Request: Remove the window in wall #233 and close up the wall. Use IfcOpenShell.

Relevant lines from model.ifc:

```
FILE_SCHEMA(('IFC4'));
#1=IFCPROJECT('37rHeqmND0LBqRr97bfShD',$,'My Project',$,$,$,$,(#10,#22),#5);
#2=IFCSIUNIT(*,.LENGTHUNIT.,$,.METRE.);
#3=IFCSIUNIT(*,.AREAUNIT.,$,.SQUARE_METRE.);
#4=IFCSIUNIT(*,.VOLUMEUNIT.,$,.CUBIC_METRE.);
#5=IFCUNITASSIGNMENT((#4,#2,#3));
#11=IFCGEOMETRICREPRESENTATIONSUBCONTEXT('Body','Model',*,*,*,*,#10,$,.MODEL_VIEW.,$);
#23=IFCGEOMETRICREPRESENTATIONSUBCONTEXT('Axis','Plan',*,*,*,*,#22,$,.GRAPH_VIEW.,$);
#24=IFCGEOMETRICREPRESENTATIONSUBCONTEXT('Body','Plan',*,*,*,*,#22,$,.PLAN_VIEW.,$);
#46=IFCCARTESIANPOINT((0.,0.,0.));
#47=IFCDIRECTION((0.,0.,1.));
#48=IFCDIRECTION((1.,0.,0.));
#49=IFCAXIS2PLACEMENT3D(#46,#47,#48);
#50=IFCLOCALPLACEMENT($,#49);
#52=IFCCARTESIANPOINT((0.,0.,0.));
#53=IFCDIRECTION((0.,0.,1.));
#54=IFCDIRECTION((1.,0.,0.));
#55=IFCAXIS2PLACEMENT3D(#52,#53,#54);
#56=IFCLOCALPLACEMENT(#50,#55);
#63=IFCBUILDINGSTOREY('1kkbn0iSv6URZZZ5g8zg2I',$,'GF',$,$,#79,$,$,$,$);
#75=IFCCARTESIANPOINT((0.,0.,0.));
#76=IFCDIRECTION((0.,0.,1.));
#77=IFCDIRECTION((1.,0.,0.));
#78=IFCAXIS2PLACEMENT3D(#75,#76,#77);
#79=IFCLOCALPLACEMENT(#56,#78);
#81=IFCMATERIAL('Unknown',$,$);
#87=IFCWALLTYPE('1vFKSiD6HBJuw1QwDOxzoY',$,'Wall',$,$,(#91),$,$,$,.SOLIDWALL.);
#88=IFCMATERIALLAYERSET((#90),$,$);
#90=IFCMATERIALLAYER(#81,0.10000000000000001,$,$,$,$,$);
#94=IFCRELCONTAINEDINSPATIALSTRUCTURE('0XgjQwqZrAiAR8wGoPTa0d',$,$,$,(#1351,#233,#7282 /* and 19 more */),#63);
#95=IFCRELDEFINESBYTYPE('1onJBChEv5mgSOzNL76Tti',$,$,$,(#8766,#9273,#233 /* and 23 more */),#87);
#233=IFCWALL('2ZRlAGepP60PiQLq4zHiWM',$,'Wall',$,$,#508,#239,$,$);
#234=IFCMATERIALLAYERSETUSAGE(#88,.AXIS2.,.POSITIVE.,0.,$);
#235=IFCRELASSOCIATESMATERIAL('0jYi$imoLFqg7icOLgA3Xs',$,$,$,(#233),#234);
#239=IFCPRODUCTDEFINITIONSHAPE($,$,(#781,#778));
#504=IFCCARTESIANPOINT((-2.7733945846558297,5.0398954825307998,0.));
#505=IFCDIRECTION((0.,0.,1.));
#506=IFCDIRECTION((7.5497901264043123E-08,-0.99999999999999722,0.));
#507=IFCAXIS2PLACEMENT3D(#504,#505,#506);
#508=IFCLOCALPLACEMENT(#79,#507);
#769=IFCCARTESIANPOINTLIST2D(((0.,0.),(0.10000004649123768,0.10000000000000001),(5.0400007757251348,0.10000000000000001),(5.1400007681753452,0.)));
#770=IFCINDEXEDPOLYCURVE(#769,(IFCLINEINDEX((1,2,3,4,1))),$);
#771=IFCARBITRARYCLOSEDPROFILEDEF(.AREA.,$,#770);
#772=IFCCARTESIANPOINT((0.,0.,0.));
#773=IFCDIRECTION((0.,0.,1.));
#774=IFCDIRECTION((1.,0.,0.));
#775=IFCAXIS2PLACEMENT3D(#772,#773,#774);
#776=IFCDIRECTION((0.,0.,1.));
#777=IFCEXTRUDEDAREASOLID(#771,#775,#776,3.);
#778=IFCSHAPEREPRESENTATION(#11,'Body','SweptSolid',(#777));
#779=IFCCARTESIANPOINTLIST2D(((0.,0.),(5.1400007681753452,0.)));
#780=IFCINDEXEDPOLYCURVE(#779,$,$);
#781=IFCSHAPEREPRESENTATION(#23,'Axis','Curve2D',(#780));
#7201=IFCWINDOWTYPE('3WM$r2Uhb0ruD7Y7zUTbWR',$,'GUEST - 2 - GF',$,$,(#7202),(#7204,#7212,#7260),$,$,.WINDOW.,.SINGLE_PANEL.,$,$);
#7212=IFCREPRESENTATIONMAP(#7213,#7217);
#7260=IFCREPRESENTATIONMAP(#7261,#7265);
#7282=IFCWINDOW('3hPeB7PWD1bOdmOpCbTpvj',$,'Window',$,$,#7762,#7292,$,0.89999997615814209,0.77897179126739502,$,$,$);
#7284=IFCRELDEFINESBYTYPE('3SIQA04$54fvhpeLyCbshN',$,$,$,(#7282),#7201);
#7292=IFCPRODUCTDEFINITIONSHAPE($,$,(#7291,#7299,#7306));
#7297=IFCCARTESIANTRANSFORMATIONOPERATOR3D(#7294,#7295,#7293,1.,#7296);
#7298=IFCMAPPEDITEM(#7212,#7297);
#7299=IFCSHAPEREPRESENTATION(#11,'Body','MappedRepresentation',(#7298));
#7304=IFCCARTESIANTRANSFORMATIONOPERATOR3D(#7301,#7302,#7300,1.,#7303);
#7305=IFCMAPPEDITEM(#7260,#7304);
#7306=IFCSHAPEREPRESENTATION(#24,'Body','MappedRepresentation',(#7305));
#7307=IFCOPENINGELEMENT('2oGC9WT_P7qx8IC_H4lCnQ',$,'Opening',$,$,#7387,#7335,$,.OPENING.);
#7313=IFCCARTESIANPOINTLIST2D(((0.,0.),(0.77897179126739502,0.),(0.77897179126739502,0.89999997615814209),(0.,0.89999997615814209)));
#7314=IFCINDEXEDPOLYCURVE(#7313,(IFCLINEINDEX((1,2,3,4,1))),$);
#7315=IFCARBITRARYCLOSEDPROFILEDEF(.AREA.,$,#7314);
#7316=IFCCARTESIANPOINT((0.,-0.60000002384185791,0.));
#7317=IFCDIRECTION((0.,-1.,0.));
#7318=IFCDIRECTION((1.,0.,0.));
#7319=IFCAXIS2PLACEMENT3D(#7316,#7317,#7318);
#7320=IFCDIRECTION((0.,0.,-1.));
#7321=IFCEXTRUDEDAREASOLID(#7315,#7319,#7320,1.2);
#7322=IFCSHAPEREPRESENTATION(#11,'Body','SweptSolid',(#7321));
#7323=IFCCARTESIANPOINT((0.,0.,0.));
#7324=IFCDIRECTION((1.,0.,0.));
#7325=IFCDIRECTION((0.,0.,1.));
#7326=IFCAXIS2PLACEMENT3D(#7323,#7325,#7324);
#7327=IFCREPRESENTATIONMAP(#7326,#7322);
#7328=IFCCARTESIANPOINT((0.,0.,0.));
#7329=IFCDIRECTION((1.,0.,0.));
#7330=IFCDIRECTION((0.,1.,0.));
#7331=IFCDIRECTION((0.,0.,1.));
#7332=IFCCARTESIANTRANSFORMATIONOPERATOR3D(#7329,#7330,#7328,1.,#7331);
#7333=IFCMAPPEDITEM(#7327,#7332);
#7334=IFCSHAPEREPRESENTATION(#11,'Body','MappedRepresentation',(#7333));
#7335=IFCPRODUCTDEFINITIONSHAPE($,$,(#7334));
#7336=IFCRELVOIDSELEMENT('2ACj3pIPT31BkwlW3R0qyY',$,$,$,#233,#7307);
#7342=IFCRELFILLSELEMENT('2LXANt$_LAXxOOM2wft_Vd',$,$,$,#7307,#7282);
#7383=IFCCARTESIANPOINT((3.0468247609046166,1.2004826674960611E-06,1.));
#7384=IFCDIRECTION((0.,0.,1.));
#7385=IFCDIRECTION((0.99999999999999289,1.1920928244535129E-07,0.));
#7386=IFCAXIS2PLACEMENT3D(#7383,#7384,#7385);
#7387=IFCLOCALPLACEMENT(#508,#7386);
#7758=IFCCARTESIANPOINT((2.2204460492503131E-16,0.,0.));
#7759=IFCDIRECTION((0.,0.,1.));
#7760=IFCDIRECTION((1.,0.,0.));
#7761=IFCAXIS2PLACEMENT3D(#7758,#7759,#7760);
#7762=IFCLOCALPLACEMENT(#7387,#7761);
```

```python
import ifcopenshell
import ifcopenshell.api.feature
import ifcopenshell.api.root
import ifcopenshell.geom
import ifcopenshell.util.shape

model = ifcopenshell.open("model.ifc")
settings = ifcopenshell.geom.settings()


def volume(element):
    """Net volume in cubic metres, openings subtracted."""
    shape = ifcopenshell.geom.create_shape(settings, element)
    return ifcopenshell.util.shape.get_volume(shape.geometry)


window = model.by_guid("3hPeB7PWD1bOdmOpCbTpvj")
opening = window.FillsVoids[0].RelatingOpeningElement
wall = opening.VoidsElements[0].RelatingBuildingElement
before = volume(wall)

ifcopenshell.api.root.remove_product(model, product=window)
ifcopenshell.api.feature.remove_feature(model, feature=opening)

after = volume(wall)

print(f"wall volume {before:.3f} -> {after:.3f} m3")

model.write("model-out.ifc")
```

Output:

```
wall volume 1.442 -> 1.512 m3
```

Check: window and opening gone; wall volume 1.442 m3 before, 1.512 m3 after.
